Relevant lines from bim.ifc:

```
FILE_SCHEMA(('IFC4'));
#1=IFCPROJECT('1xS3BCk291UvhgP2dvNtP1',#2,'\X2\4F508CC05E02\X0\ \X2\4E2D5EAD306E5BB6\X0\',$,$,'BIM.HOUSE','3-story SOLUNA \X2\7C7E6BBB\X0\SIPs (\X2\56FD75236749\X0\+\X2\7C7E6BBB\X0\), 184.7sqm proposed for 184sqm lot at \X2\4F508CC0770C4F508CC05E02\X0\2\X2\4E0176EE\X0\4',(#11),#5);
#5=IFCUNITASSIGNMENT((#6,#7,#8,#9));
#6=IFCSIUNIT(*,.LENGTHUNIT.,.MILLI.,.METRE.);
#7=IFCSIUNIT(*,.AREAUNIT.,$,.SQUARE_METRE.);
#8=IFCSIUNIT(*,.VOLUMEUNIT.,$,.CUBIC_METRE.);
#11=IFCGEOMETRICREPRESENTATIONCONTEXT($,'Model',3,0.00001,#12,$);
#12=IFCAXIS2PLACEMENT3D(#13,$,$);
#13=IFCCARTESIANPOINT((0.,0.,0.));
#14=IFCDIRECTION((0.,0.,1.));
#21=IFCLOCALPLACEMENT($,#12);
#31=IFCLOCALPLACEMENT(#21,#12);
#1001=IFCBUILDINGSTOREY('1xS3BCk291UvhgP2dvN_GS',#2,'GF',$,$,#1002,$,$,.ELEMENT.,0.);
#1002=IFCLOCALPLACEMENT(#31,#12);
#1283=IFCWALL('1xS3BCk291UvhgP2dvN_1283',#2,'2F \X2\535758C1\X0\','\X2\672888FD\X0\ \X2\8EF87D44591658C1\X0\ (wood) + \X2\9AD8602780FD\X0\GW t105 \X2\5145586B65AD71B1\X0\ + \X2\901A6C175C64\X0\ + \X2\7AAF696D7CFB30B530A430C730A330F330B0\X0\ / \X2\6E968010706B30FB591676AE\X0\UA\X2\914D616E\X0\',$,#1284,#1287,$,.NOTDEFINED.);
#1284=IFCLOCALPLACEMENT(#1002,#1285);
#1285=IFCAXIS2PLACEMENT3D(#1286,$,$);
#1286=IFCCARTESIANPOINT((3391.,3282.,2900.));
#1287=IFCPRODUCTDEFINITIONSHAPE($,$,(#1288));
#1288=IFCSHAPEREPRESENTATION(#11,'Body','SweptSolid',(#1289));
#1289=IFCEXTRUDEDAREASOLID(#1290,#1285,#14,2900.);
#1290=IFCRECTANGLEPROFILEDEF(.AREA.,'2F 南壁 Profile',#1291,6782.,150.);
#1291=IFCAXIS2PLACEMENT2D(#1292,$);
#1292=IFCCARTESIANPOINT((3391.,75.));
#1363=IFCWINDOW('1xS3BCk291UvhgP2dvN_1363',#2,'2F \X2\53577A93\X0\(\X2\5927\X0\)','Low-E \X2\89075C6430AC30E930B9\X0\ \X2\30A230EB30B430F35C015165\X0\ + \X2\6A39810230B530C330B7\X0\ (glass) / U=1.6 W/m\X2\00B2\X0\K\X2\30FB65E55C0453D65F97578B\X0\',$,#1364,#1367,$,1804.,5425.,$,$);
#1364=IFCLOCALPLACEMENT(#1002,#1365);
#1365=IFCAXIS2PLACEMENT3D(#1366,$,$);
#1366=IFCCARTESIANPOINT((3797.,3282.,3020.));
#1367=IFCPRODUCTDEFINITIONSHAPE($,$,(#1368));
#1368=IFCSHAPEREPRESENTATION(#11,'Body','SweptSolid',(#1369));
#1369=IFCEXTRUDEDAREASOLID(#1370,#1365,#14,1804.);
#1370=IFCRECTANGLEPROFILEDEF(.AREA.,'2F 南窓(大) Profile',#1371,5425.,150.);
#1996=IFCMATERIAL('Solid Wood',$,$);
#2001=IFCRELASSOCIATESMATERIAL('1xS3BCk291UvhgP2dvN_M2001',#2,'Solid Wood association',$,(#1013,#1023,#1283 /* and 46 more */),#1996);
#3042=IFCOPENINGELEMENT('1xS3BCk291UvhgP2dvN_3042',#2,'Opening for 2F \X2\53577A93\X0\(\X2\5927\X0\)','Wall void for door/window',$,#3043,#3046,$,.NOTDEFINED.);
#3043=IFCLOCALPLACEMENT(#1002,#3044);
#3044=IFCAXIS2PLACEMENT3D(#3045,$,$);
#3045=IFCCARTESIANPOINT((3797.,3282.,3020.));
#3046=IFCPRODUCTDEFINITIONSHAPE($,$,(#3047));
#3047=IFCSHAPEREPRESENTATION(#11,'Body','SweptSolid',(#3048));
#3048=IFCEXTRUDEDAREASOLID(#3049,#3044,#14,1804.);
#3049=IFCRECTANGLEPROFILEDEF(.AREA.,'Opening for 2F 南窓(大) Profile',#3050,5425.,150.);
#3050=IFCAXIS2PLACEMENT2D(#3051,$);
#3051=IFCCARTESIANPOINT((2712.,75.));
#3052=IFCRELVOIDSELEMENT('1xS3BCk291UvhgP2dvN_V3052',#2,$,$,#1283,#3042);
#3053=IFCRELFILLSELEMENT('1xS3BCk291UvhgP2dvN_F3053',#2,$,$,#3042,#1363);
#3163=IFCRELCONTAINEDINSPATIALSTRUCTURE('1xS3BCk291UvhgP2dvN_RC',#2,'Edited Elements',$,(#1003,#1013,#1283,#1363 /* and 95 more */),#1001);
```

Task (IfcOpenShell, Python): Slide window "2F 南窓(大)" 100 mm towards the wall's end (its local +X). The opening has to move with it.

```python
import ifcopenshell
import ifcopenshell.api.geometry
import ifcopenshell.util.placement

model = ifcopenshell.open("bim.ifc")

window = model.by_guid("1xS3BCk291UvhgP2dvN_1363")
opening = window.FillsVoids[0].RelatingOpeningElement
wall = opening.VoidsElements[0].RelatingBuildingElement

wall_matrix = ifcopenshell.util.placement.get_local_placement(wall.ObjectPlacement)
shift = wall_matrix[:3, 0] * 100.0
before = ifcopenshell.util.placement.get_local_placement(window.ObjectPlacement)[:3, 3].copy()

# The window is not placed relative to its opening, so move both.
for product in (opening, window):
    matrix = ifcopenshell.util.placement.get_local_placement(product.ObjectPlacement)
    matrix[:3, 3] += shift
    ifcopenshell.api.geometry.edit_object_placement(model, product=product, matrix=matrix, is_si=False)

after = ifcopenshell.util.placement.get_local_placement(window.ObjectPlacement)[:3, 3]
print("window moved by", (after - before).round(3) + 0.0)

model.write("bim_rev.ifc")
```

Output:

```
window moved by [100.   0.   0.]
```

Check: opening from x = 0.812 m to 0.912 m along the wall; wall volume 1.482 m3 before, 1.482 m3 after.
